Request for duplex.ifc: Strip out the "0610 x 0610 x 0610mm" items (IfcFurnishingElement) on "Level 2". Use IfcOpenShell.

First a look at what the model holds.

```python
import ifcopenshell
import ifcopenshell.util.element

model = ifcopenshell.open("duplex.ifc")
print(model.schema)
storey = next(s for s in model.by_type("IfcBuildingStorey") if s.Name == "Level 2")
furniture = [e for e in ifcopenshell.util.element.get_decomposition(storey) if e.is_a("IfcFurnishingElement")]
seen = {}
for e in furniture:
    element_type = ifcopenshell.util.element.get_type(e)
    name = element_type.Name if element_type not in (None, e) else None
    seen[name] = seen.get(name, 0) + 1
for name, count in sorted(seen.items(), key=str):
    print(count, "x", name)
```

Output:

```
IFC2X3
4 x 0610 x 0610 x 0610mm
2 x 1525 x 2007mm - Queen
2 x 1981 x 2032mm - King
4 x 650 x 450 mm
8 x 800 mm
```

```python
import ifcopenshell
import ifcopenshell.api.root
import ifcopenshell.util.element

model = ifcopenshell.open("duplex.ifc")

storey = next(s for s in model.by_type("IfcBuildingStorey") if s.Name == "Level 2")
furniture = [e for e in ifcopenshell.util.element.get_decomposition(storey) if e.is_a("IfcFurnishingElement")]
targets = [e for e in furniture if (t := ifcopenshell.util.element.get_type(e)) not in (None, e) and t.Name == "0610 x 0610 x 0610mm"]

for e in targets:
    ifcopenshell.api.root.remove_product(model, product=e)
print(len(targets), "removed")

model.write("duplex_rev.ifc")
```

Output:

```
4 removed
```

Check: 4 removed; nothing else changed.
